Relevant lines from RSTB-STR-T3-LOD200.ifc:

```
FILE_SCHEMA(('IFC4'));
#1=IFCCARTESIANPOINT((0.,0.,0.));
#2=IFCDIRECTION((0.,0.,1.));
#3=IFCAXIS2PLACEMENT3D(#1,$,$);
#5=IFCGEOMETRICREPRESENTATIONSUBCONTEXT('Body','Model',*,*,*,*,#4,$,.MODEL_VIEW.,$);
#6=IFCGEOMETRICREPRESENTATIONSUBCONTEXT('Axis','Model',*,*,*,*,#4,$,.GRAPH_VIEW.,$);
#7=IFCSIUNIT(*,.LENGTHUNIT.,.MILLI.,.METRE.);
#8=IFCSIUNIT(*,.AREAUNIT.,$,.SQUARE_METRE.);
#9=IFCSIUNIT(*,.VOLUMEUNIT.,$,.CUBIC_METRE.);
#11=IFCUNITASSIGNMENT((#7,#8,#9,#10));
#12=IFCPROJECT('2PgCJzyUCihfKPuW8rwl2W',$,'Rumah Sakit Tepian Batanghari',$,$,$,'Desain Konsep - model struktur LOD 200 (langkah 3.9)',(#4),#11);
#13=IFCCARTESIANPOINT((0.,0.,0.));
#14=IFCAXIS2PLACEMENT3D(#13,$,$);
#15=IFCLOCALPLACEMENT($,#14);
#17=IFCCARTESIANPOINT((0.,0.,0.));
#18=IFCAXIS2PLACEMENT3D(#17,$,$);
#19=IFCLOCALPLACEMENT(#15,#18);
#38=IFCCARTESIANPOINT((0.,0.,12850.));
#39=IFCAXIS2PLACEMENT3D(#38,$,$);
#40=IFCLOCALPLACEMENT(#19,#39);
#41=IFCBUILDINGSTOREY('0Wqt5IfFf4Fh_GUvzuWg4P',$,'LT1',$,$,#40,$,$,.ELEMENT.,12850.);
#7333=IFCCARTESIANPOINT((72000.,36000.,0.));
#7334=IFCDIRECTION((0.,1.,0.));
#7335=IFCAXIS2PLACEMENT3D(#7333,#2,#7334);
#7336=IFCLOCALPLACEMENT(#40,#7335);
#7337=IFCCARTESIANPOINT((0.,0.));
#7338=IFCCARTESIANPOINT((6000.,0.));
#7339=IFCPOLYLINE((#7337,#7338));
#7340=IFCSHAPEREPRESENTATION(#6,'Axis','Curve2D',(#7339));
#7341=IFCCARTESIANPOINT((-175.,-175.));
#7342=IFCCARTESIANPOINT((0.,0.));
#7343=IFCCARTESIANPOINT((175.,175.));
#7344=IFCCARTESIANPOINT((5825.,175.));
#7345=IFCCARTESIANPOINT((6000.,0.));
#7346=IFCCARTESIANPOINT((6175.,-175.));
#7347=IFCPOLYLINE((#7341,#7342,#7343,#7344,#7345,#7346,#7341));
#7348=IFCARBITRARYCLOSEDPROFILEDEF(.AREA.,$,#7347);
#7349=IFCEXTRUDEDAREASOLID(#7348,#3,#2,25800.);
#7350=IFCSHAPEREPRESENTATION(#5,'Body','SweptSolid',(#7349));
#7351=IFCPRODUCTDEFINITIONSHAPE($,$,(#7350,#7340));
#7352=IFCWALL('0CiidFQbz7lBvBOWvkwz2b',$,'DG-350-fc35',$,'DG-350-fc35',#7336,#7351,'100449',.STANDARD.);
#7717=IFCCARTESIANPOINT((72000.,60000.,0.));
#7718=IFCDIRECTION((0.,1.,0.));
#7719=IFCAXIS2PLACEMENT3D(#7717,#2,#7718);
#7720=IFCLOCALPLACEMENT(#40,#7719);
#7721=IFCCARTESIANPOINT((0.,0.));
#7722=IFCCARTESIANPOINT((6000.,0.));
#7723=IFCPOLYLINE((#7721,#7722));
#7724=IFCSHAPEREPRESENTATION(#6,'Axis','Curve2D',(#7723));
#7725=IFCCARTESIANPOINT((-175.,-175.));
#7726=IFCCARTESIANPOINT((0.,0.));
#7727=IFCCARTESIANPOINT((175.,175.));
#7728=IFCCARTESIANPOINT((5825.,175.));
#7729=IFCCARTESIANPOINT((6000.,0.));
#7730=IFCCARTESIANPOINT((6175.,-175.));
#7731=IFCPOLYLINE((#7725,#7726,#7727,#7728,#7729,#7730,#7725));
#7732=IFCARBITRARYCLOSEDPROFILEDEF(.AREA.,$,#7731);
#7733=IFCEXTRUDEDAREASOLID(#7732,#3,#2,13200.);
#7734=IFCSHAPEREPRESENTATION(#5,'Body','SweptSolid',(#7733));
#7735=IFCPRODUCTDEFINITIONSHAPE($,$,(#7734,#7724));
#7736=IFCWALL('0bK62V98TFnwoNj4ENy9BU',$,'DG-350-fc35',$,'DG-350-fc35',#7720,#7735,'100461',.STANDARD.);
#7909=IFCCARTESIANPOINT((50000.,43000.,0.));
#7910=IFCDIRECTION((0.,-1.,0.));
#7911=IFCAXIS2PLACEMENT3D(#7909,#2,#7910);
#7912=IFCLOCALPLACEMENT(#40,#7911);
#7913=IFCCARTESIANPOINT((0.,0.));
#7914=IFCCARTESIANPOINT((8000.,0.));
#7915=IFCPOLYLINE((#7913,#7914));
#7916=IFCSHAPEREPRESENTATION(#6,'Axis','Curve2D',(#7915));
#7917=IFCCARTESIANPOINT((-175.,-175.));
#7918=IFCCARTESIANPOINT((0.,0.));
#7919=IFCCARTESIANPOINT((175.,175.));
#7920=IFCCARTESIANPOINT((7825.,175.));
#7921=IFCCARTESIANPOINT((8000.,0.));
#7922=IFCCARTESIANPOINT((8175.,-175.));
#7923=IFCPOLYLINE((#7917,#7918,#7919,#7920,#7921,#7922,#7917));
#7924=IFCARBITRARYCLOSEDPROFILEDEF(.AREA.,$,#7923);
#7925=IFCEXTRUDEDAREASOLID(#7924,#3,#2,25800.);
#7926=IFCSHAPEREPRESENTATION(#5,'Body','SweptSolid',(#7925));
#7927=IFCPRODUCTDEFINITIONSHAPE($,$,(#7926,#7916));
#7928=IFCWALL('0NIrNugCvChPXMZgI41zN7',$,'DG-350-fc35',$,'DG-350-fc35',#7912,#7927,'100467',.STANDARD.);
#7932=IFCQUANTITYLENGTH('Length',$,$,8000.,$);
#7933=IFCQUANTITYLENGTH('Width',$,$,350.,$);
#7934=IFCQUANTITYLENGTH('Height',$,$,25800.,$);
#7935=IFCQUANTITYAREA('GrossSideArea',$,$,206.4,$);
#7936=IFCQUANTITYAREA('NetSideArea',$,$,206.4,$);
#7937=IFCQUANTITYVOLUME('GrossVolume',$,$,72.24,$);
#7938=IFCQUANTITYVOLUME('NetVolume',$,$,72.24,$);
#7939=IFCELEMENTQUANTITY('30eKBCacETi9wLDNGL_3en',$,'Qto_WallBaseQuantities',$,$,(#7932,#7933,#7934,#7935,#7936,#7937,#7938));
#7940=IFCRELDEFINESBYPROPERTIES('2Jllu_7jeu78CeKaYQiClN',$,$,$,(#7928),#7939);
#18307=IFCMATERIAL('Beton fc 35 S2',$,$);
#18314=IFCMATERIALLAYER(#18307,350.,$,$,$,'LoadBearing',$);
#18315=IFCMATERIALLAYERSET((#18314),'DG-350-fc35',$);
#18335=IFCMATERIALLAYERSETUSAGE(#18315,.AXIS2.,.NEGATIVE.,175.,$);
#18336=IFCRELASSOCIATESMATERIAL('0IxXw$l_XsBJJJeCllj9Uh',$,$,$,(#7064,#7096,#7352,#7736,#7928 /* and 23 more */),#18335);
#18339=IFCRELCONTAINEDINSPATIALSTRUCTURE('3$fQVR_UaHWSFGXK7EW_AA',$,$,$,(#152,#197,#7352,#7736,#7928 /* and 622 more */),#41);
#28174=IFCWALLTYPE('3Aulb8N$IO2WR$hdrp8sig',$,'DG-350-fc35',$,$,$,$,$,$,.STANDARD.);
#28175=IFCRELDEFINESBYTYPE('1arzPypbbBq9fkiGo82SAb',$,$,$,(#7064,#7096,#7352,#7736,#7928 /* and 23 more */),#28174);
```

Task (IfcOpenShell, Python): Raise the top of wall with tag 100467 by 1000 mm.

```python
import ifcopenshell
import ifcopenshell.api.pset
import ifcopenshell.geom
import ifcopenshell.util.element
import ifcopenshell.util.representation
import ifcopenshell.util.shape
import ifcopenshell.util.unit

model = ifcopenshell.open("RSTB-STR-T3-LOD200.ifc")
unit_scale = ifcopenshell.util.unit.calculate_unit_scale(model)
area_scale = ifcopenshell.util.unit.calculate_unit_scale(model, "AREAUNIT")
volume_scale = ifcopenshell.util.unit.calculate_unit_scale(model, "VOLUMEUNIT")
settings = ifcopenshell.geom.settings()


def volume(element):
    """Net volume in cubic metres, openings subtracted."""
    shape = ifcopenshell.geom.create_shape(settings, element)
    return ifcopenshell.util.shape.get_volume(shape.geometry)


wall = model.by_id(7928)
before = volume(wall)

body = ifcopenshell.util.representation.get_representation(wall, "Model", "Body")
solid = body.Items[0]
old_height = solid.Depth
solid.Depth += 1000.0
after = volume(wall)
thickness = 0.35  # wall thickness in metres

# Update the stored height, areas and volumes.
qto = model.by_id(ifcopenshell.util.element.get_pset(wall, "Qto_WallBaseQuantities", should_inherit=False)["id"])
ifcopenshell.api.pset.edit_qto(model, qto=qto, properties={
    "Height": solid.Depth,
    "GrossSideArea": ifcopenshell.util.element.get_pset(wall, "Qto_WallBaseQuantities", "GrossSideArea") * solid.Depth / old_height,
    "NetSideArea": after / thickness / area_scale,
    "GrossVolume": ifcopenshell.util.element.get_pset(wall, "Qto_WallBaseQuantities", "GrossVolume") * solid.Depth / old_height,
    "NetVolume": after / volume_scale,
})

print(f"height {old_height:g} -> {solid.Depth:g}, volume {before:.3f} -> {after:.3f} m3")

model.write("RSTB-STR-T3-LOD200_rev.ifc")
```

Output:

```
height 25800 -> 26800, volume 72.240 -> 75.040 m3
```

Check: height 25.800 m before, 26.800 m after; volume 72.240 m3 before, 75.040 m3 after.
